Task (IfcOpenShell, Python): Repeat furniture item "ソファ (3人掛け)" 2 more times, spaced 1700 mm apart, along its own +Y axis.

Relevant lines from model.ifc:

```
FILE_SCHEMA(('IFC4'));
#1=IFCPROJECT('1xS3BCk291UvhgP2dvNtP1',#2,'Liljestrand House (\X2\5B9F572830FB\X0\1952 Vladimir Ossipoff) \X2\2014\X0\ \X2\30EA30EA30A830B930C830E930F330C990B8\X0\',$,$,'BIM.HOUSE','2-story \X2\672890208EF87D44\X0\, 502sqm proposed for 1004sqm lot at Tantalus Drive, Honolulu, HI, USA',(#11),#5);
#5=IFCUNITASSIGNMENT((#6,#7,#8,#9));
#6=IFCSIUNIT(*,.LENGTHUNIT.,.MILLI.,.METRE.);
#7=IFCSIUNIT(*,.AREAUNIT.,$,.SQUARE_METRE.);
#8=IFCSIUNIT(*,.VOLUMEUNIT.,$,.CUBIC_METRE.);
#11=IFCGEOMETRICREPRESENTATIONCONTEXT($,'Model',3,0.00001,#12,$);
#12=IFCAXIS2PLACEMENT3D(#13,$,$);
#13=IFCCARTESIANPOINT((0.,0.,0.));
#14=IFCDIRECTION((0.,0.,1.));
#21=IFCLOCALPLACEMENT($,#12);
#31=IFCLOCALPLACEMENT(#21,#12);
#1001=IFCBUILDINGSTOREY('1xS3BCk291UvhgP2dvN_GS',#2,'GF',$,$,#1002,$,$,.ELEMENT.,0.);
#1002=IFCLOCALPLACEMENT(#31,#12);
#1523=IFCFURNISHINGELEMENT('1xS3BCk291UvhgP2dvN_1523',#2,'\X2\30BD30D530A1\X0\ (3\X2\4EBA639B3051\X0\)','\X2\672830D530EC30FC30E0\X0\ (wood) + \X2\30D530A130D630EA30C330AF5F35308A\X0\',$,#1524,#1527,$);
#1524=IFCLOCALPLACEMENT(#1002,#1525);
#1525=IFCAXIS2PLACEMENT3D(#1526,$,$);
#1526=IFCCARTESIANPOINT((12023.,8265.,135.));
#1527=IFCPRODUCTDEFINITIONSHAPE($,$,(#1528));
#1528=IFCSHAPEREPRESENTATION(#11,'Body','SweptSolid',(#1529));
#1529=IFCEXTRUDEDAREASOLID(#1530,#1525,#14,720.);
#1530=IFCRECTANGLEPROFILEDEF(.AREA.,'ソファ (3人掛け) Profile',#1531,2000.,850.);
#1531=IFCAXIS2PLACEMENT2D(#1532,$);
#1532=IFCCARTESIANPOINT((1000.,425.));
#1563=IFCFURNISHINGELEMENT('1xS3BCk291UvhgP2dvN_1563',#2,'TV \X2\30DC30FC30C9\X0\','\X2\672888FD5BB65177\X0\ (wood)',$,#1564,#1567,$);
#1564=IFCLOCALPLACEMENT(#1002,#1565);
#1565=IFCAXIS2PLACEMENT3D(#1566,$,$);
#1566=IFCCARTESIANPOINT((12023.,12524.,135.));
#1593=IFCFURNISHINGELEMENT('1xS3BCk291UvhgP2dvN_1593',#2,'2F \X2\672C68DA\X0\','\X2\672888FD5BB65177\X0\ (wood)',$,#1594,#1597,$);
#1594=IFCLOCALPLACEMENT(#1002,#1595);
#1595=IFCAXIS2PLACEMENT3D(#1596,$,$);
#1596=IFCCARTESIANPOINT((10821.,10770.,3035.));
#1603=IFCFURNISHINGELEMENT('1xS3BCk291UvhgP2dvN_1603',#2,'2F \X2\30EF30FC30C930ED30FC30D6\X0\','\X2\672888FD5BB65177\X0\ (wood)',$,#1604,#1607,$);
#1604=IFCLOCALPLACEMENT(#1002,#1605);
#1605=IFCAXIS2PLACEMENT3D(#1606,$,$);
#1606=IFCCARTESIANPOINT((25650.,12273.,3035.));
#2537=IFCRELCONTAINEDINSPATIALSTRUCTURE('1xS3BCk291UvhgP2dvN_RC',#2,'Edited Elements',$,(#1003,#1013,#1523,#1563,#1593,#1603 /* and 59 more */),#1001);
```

```python
import ifcopenshell
import ifcopenshell.api.geometry
import ifcopenshell.api.root
import ifcopenshell.util.element
import ifcopenshell.util.placement
import ifcopenshell.util.unit

model = ifcopenshell.open("model.ifc")
unit_scale = ifcopenshell.util.unit.calculate_unit_scale(model)


def reuse_history(source, copy):
    """copy_class also copies each property set's owner history, people and application; keep the originals."""
    for rel in copy.IsDefinedBy:
        if rel.is_a("IfcRelDefinesByProperties") and (history := rel.RelatingPropertyDefinition.OwnerHistory):
            rel.RelatingPropertyDefinition.OwnerHistory = source.OwnerHistory
            ifcopenshell.util.element.remove_deep2(model, history)


source = model.by_guid("1xS3BCk291UvhgP2dvN_1523")
base = ifcopenshell.util.placement.get_local_placement(source.ObjectPlacement)
step = base[:3, 1] * 1.7 / unit_scale

for i in range(1, 3):
    copy = ifcopenshell.api.root.copy_class(model, product=source)
    copy.Representation = ifcopenshell.util.element.copy_deep(
        model, source.Representation, exclude=["IfcGeometricRepresentationContext", "IfcRepresentationMap"]
    )
    reuse_history(source, copy)
    matrix = base.copy()
    matrix[:3, 3] += i * step
    print("added at", matrix[:3, 3].round(3) + 0.0)
    ifcopenshell.api.geometry.edit_object_placement(model, product=copy, matrix=matrix, is_si=False)

model.write("model_rev.ifc")
```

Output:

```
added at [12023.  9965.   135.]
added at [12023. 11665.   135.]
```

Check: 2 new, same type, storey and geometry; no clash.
